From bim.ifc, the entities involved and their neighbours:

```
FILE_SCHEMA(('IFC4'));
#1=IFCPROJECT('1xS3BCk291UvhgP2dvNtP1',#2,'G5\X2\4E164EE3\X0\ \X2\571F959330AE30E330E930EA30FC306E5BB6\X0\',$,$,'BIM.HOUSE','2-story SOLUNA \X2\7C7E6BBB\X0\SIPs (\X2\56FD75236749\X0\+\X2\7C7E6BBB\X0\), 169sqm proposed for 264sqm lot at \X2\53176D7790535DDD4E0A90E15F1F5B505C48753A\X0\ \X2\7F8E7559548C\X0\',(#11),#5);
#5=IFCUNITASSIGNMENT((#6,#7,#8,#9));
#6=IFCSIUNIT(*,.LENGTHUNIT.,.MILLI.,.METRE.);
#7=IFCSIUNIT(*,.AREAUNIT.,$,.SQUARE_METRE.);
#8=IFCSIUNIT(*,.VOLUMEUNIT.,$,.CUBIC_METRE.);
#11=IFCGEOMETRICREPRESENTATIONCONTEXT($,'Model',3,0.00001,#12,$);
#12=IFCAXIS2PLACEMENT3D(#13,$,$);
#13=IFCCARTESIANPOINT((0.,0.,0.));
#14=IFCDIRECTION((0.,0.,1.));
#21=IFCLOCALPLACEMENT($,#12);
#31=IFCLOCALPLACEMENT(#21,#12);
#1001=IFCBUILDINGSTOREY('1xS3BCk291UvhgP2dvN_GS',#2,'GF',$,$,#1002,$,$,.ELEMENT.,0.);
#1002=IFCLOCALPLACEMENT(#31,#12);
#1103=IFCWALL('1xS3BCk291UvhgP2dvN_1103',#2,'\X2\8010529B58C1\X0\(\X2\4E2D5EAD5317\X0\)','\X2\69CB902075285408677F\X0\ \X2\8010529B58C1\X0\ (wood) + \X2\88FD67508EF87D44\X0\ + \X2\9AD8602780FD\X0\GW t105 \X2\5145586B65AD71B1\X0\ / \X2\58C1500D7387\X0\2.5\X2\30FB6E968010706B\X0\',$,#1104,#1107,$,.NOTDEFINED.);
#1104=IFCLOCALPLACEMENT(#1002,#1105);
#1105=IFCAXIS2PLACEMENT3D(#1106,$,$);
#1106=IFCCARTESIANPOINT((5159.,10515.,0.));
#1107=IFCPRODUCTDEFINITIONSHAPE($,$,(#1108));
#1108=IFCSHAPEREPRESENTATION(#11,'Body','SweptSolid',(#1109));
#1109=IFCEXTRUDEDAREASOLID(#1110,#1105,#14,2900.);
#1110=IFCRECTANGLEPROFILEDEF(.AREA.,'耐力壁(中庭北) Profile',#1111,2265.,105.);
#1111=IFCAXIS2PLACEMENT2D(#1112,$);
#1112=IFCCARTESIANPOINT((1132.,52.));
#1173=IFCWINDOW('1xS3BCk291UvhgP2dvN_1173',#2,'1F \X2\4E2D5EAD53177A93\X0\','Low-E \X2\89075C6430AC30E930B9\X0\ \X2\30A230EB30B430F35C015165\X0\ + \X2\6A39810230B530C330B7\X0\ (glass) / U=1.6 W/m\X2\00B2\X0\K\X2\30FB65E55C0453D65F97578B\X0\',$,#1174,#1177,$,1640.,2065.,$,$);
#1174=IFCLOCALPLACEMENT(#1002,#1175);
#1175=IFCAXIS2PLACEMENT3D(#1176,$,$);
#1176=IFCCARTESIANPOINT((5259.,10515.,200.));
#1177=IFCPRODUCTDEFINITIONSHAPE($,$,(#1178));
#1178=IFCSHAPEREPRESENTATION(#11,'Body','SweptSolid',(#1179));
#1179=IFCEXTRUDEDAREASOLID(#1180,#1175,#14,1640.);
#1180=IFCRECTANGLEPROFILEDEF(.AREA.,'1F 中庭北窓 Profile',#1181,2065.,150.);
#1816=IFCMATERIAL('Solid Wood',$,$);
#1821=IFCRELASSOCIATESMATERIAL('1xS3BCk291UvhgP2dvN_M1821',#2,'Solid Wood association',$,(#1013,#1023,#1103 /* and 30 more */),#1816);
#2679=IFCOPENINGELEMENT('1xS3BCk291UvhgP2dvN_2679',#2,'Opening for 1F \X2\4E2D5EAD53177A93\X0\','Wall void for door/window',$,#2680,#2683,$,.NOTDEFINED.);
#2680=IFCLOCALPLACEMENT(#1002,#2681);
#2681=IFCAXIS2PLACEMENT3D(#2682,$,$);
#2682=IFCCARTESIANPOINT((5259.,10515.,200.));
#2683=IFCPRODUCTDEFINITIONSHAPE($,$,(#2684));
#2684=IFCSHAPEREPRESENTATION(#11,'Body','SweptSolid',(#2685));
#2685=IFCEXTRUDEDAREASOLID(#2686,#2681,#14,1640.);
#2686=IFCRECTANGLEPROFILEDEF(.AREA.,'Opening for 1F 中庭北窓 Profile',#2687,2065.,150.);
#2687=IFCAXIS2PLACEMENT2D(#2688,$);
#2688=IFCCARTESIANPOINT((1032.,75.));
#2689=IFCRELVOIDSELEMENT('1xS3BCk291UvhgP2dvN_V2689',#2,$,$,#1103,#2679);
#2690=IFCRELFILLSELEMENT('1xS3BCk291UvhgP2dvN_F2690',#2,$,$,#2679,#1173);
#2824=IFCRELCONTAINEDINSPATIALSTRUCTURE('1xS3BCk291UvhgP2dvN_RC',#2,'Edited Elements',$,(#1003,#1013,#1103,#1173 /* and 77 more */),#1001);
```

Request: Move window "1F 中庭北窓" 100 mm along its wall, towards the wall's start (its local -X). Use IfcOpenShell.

```python
import ifcopenshell
import ifcopenshell.api.geometry
import ifcopenshell.util.placement

model = ifcopenshell.open("bim.ifc")

window = model.by_guid("1xS3BCk291UvhgP2dvN_1173")
opening = window.FillsVoids[0].RelatingOpeningElement
wall = opening.VoidsElements[0].RelatingBuildingElement

wall_matrix = ifcopenshell.util.placement.get_local_placement(wall.ObjectPlacement)
shift = wall_matrix[:3, 0] * -100.0
before = ifcopenshell.util.placement.get_local_placement(window.ObjectPlacement)[:3, 3].copy()

# The window is not placed relative to its opening, so move both.
for product in (opening, window):
    matrix = ifcopenshell.util.placement.get_local_placement(product.ObjectPlacement)
    matrix[:3, 3] += shift
    ifcopenshell.api.geometry.edit_object_placement(model, product=product, matrix=matrix, is_si=False)

after = ifcopenshell.util.placement.get_local_placement(window.ObjectPlacement)[:3, 3]
print("window moved by", (after - before).round(3) + 0.0)

model.write("bim_edited.ifc")
```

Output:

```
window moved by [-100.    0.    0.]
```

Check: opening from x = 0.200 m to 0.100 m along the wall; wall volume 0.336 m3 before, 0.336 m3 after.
